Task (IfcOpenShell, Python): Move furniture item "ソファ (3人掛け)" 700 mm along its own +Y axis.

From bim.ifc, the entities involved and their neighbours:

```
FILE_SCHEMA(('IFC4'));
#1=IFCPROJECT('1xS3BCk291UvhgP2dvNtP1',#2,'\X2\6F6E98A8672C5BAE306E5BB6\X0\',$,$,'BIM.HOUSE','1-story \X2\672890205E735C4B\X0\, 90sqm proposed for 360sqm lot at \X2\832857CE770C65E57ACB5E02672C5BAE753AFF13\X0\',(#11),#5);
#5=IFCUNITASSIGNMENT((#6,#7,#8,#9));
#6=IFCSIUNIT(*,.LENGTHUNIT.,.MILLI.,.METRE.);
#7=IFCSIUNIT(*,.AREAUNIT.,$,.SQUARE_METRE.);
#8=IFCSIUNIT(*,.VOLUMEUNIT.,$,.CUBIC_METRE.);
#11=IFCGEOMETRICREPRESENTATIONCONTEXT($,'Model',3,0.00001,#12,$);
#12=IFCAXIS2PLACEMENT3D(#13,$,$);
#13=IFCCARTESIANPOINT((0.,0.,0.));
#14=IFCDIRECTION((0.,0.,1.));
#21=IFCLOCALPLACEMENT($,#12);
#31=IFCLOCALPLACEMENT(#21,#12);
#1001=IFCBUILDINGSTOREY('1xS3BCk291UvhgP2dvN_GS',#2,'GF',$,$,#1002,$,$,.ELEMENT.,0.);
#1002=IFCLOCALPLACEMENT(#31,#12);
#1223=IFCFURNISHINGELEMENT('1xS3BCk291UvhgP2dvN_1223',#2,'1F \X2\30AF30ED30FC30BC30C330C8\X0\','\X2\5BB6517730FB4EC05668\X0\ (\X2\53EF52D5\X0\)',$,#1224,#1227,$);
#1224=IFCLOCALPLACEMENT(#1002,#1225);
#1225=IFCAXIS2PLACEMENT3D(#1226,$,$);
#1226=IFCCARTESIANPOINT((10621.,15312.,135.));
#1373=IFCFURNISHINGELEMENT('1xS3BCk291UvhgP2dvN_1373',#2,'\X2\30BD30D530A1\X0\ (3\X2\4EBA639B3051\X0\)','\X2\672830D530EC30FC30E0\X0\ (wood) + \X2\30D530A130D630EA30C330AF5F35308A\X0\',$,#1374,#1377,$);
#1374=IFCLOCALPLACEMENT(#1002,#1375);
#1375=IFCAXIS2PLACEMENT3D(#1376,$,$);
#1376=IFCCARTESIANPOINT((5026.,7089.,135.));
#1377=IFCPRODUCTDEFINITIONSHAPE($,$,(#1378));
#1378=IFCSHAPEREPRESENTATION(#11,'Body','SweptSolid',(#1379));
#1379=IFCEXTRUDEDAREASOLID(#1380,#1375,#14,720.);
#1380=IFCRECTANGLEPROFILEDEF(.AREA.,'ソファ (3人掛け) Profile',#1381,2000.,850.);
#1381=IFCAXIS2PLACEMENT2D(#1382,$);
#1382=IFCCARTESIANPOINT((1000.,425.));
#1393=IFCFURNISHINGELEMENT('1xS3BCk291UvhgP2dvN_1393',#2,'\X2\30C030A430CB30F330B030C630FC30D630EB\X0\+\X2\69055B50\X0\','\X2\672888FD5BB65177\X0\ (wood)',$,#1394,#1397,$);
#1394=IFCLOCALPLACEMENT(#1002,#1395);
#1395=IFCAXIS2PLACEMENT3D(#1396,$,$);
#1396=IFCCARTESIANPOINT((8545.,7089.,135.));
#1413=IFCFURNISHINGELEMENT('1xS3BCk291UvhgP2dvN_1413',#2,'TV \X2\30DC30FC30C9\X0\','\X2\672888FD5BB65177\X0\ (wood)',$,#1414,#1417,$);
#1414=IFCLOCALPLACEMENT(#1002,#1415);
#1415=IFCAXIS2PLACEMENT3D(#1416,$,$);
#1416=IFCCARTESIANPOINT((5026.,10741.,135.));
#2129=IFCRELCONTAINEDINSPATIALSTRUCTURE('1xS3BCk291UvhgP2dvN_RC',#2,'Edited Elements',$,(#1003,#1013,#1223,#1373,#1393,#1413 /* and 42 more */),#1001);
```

```python
import ifcopenshell
import ifcopenshell.api.geometry
import ifcopenshell.util.placement
import ifcopenshell.util.unit

model = ifcopenshell.open("bim.ifc")
unit_scale = ifcopenshell.util.unit.calculate_unit_scale(model)

item = model.by_guid("1xS3BCk291UvhgP2dvN_1373")
matrix = ifcopenshell.util.placement.get_local_placement(item.ObjectPlacement)
matrix[:3, 3] += matrix[:3, 1] * 0.7 / unit_scale
ifcopenshell.api.geometry.edit_object_placement(model, product=item, matrix=matrix, is_si=False)

print(ifcopenshell.util.placement.get_local_placement(item.ObjectPlacement).round(3) + 0.0)

model.write("bim_rev.ifc")
```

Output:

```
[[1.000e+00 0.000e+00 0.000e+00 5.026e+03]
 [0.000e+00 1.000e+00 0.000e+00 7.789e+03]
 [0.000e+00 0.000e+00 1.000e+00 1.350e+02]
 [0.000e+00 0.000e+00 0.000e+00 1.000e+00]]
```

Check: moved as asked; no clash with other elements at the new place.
